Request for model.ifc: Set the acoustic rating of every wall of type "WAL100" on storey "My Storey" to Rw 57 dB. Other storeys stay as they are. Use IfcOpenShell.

First a look at what the model holds.

```python
import ifcopenshell
import ifcopenshell.util.element

model = ifcopenshell.open("model.ifc")
print(model.schema)
storey = next(s for s in model.by_type("IfcBuildingStorey") if s.Name == "My Storey")
walls = [e for e in ifcopenshell.util.element.get_decomposition(storey) if e.is_a("IfcWall")]
seen = {}
for e in walls:
    element_type = ifcopenshell.util.element.get_type(e)
    key = (element_type.Name if element_type != e and element_type else None, ifcopenshell.util.element.get_pset(e, "Pset_WallCommon", "AcousticRating"))
    seen[key] = seen.get(key, 0) + 1
for (name, value), count in sorted(seen.items(), key=str):
    print(count, "x", name, "|", value)
```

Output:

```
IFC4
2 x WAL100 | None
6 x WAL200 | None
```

```python
import ifcopenshell
import ifcopenshell.api.pset
import ifcopenshell.util.element

model = ifcopenshell.open("model.ifc")

storey = next(s for s in model.by_type("IfcBuildingStorey") if s.Name == "My Storey")
walls = [e for e in ifcopenshell.util.element.get_decomposition(storey) if e.is_a("IfcWall")]

count = 0
for e in walls:
    element_type = ifcopenshell.util.element.get_type(e)
    if element_type in (None, e) or element_type.Name != "WAL100":
        continue
    # add_pset returns the element's existing set when there is one.
    pset = ifcopenshell.api.pset.add_pset(model, product=e, name="Pset_WallCommon")
    ifcopenshell.api.pset.edit_pset(model, pset=pset, properties={"AcousticRating": "Rw 57 dB"})
    count += 1

print(count, "walls updated")

model.write("model_v2.ifc")
```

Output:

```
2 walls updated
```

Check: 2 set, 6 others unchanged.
